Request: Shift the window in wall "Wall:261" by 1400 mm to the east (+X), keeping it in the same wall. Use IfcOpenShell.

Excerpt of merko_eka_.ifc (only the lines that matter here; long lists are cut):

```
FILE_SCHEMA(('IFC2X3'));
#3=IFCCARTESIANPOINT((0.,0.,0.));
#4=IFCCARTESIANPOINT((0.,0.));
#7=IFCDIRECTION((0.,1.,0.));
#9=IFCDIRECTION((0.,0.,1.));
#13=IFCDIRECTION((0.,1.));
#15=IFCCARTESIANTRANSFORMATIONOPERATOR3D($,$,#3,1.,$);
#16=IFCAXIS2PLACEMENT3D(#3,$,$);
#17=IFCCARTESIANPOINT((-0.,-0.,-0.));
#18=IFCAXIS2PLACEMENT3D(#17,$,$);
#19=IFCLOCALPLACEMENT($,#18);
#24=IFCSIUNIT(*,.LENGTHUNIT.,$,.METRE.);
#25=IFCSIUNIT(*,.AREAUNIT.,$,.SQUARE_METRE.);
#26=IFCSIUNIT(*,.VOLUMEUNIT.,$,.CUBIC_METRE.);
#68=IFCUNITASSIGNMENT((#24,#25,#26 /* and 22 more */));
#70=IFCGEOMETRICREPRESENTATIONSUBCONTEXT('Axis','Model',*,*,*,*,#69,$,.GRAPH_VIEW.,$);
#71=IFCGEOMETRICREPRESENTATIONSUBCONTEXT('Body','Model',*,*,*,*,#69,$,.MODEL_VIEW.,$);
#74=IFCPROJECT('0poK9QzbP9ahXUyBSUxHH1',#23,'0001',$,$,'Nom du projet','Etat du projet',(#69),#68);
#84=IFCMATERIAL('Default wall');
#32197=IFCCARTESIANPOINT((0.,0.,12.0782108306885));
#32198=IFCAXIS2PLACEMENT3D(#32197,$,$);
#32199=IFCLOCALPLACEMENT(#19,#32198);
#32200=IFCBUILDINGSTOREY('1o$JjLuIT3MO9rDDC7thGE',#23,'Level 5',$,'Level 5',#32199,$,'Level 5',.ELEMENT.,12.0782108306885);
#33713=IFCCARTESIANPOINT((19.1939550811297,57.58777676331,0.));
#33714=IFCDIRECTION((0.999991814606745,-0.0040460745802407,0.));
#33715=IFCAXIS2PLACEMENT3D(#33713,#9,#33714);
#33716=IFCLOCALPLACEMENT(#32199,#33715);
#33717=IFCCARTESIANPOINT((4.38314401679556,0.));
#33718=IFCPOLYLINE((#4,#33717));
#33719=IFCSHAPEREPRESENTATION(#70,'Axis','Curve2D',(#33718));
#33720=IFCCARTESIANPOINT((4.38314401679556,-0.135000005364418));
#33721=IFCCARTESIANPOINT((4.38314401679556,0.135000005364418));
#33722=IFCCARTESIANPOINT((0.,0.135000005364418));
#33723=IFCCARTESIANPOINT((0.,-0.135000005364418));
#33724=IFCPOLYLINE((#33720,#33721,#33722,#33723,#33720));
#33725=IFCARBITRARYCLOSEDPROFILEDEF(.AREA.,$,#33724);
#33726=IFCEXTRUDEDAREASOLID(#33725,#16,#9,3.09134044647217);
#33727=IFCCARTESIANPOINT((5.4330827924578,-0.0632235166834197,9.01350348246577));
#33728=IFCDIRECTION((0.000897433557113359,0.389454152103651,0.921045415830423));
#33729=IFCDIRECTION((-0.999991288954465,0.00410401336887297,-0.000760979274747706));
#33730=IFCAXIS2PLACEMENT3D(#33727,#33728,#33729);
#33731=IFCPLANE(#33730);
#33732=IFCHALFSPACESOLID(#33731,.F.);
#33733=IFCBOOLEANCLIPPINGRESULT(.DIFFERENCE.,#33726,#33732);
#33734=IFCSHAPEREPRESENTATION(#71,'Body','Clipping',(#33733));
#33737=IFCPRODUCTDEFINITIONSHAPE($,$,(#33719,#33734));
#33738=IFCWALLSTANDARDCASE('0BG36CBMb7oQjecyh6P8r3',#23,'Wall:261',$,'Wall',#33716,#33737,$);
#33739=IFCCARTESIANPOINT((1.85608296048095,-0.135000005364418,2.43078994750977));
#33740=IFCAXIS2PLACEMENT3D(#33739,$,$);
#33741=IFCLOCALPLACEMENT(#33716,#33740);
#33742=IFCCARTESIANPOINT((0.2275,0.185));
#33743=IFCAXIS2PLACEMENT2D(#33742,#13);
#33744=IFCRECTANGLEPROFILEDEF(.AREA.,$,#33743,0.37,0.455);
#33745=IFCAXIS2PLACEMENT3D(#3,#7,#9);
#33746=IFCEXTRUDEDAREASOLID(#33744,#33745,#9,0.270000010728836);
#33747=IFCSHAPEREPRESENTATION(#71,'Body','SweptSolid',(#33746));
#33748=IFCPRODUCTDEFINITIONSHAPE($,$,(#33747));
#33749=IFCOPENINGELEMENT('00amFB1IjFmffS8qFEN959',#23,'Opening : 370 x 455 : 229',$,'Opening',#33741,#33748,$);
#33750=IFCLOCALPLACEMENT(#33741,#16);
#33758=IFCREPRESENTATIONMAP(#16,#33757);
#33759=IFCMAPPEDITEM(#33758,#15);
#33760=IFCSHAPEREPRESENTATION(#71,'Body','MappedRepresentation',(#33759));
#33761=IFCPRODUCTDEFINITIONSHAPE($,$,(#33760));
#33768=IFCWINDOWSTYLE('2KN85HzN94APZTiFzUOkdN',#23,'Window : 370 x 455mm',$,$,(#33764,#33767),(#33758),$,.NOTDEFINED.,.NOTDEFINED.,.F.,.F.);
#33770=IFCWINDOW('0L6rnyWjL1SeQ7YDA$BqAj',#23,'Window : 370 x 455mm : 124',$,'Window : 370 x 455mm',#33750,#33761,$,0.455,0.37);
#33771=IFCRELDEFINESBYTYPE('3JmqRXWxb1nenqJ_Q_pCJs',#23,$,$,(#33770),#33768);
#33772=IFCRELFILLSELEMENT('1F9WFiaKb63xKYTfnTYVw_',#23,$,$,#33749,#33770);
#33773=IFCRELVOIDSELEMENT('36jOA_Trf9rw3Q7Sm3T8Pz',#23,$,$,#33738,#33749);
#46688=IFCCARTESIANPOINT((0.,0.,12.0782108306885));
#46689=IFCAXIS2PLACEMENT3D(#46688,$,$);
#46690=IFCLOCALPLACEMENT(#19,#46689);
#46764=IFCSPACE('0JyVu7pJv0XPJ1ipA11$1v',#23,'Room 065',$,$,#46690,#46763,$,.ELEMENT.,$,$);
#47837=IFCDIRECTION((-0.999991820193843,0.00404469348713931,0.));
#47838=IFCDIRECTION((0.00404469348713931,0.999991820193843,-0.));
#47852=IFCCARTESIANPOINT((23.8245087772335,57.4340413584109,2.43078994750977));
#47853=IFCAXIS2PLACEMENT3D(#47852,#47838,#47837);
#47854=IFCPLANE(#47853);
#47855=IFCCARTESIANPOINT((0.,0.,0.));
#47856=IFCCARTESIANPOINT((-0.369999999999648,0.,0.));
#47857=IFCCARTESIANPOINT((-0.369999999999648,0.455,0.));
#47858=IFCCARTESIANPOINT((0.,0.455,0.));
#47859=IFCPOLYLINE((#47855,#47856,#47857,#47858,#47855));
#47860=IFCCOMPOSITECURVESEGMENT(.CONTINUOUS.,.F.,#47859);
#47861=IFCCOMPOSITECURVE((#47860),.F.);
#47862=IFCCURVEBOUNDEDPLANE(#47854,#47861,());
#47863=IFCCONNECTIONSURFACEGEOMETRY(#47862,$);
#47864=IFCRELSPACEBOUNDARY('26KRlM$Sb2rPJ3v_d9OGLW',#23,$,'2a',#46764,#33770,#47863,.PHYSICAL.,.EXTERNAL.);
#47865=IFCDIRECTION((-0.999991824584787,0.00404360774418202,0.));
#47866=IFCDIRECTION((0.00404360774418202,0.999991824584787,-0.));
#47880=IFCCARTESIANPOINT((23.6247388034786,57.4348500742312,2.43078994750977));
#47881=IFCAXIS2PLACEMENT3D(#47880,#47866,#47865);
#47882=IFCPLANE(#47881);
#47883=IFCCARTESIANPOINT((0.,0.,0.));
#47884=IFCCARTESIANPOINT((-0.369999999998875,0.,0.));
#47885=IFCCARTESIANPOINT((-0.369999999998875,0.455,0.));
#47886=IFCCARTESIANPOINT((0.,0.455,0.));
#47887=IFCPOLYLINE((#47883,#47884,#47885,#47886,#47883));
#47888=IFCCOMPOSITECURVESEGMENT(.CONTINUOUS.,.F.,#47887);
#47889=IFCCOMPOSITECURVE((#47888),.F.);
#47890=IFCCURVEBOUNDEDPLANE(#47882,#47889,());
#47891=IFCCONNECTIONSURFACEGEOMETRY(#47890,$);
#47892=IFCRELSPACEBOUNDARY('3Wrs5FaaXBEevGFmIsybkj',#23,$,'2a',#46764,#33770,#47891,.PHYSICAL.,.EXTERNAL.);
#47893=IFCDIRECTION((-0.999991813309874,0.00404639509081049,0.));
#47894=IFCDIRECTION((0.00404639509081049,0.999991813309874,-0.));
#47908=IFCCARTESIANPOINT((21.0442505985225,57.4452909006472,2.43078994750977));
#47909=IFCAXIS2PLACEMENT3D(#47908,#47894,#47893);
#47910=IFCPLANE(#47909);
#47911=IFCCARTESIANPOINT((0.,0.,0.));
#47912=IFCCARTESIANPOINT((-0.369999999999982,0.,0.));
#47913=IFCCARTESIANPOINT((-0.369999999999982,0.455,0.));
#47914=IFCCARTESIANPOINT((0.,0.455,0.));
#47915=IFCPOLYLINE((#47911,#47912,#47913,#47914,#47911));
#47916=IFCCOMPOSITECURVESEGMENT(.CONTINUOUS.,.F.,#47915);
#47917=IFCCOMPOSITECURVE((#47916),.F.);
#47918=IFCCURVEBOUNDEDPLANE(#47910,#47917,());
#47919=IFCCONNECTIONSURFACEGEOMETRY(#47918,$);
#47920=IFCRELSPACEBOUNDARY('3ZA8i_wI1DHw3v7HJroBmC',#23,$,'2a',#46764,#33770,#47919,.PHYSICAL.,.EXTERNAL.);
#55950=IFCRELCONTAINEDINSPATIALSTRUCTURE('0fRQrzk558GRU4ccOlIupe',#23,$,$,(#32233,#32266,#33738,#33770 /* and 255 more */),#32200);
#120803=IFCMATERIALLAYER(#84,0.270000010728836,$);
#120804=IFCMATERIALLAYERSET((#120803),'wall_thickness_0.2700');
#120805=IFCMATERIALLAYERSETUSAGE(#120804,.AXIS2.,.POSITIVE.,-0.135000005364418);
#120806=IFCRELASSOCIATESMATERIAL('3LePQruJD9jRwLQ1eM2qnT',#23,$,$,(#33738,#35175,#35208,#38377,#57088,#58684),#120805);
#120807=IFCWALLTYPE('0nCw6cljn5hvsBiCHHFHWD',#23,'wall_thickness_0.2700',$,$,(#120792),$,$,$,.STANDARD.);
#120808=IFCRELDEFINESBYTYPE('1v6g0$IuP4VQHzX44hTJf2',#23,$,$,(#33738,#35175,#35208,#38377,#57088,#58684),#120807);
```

```python
import numpy as np
import ifcopenshell
import ifcopenshell.api.geometry
import ifcopenshell.util.placement
import ifcopenshell.util.unit

model = ifcopenshell.open("merko_eka_.ifc")
unit_scale = ifcopenshell.util.unit.calculate_unit_scale(model)

window = model.by_guid("0L6rnyWjL1SeQ7YDA$BqAj")
opening = window.FillsVoids[0].RelatingOpeningElement
wall = opening.VoidsElements[0].RelatingBuildingElement

wall_matrix = ifcopenshell.util.placement.get_local_placement(wall.ObjectPlacement)
shift = wall_matrix[:3, 0] * 1.4 / unit_scale
before = ifcopenshell.util.placement.get_local_placement(window.ObjectPlacement)[:3, 3].copy()

# The window is placed relative to its opening, so it follows when the opening moves.
matrix = ifcopenshell.util.placement.get_local_placement(opening.ObjectPlacement)
matrix[:3, 3] += shift
ifcopenshell.api.geometry.edit_object_placement(
    model, product=opening, matrix=matrix, is_si=False, should_transform_children=True
)

# Space boundary surfaces are stored in each space's coordinates; move them too.
for rel in window.ProvidesBoundaries:
    if not rel.ConnectionGeometry:
        continue
    surface = rel.ConnectionGeometry.SurfaceOnRelatingElement.BasisSurface
    space_matrix = ifcopenshell.util.placement.get_local_placement(rel.RelatingSpace.ObjectPlacement)
    point = np.array(surface.Position.Location.Coordinates) + space_matrix[:3, :3].T @ shift
    surface.Position = model.createIfcAxis2Placement3D(
        model.createIfcCartesianPoint(point.tolist()), surface.Position.Axis, surface.Position.RefDirection
    )

after = ifcopenshell.util.placement.get_local_placement(window.ObjectPlacement)[:3, 3]
print("window moved by", (after - before).round(3) + 0.0)

model.write("merko_eka__edited.ifc")
```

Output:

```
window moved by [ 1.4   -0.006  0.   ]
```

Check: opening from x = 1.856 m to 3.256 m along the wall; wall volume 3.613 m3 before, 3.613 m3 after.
